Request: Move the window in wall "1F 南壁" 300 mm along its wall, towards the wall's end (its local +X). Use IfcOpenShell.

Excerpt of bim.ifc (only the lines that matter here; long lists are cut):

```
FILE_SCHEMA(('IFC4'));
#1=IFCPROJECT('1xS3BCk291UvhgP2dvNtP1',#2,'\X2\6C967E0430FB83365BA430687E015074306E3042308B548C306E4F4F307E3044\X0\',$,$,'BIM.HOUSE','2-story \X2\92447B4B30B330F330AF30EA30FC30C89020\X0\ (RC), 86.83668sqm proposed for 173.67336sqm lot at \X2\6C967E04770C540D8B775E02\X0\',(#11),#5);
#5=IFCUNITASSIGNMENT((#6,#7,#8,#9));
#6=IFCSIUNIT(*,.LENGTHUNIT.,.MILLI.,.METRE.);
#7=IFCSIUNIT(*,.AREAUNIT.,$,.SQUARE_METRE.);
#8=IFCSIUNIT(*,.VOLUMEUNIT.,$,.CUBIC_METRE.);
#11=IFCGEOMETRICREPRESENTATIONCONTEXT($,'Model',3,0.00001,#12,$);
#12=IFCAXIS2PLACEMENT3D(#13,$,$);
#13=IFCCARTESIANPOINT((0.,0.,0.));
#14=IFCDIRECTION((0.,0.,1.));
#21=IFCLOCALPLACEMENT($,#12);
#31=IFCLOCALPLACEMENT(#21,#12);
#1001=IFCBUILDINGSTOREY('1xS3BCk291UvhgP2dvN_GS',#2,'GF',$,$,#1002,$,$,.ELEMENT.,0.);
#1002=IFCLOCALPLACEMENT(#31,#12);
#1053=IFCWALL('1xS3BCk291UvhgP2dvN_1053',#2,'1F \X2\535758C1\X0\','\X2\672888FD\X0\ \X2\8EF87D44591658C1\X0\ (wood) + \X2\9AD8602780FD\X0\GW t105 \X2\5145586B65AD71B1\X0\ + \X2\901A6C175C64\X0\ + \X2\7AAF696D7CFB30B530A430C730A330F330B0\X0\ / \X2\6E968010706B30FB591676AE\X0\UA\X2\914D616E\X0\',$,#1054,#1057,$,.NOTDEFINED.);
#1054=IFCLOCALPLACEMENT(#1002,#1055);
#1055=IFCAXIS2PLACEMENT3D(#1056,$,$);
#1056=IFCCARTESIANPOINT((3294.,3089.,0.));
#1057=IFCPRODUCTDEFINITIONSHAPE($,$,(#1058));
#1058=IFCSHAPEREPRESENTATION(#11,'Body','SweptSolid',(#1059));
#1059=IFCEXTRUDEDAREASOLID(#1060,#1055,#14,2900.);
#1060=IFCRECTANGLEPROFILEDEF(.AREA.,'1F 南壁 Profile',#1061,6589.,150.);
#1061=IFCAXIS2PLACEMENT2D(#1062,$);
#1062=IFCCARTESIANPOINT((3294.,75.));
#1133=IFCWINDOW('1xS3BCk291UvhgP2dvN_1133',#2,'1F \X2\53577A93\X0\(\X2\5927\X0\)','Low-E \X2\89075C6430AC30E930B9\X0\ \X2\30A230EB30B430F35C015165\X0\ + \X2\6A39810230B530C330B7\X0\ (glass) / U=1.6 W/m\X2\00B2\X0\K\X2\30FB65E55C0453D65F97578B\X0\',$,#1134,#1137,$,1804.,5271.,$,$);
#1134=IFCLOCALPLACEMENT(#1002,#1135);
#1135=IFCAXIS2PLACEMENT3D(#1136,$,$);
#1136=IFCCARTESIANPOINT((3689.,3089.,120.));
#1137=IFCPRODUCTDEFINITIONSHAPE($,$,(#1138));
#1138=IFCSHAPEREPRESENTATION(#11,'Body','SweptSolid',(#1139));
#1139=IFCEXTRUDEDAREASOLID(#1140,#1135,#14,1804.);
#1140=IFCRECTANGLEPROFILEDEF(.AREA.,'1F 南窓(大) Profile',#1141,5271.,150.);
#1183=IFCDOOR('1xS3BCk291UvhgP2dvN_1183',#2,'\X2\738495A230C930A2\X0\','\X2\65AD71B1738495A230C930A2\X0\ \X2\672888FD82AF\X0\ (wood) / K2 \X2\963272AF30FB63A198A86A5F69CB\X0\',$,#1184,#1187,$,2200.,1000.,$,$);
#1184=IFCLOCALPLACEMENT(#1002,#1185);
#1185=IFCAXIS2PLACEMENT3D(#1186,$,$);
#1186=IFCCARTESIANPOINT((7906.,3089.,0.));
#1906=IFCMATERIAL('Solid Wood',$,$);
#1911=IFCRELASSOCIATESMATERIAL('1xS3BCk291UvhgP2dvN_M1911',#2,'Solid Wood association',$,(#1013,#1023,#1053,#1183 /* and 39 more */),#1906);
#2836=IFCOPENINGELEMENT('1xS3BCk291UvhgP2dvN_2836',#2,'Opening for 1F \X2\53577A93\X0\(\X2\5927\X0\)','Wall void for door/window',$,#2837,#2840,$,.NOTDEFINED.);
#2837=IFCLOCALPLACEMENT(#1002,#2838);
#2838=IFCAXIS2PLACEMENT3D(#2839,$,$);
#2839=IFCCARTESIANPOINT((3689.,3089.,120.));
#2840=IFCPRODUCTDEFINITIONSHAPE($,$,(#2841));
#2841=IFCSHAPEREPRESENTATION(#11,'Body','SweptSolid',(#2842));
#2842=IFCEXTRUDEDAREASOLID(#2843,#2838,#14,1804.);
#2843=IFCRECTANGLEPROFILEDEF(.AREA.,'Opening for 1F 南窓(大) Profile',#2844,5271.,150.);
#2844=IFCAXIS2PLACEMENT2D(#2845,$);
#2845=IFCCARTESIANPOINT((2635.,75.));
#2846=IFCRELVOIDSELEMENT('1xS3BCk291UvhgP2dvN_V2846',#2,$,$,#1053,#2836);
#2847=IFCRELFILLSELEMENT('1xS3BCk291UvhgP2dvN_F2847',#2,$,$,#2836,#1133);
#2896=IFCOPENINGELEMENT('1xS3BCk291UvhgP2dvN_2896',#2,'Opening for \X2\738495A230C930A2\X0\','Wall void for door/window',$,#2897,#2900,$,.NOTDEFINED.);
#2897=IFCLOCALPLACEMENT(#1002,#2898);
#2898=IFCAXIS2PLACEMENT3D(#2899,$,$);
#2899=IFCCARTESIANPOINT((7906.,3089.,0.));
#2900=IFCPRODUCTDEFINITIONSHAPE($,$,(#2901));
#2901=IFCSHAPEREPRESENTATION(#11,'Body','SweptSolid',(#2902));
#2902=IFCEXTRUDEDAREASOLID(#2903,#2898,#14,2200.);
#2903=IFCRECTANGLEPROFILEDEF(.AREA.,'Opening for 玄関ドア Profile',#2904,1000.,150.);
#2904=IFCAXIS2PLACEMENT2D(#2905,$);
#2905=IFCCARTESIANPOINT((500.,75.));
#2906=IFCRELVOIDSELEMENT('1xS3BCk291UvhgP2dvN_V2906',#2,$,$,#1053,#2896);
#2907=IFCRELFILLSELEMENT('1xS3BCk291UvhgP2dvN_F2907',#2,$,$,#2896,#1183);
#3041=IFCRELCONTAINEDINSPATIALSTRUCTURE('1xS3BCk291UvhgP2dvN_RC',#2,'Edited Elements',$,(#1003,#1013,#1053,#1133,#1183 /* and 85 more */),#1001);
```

```python
import ifcopenshell
import ifcopenshell.api.geometry
import ifcopenshell.util.placement
import ifcopenshell.util.unit

model = ifcopenshell.open("bim.ifc")
unit_scale = ifcopenshell.util.unit.calculate_unit_scale(model)

window = model.by_guid("1xS3BCk291UvhgP2dvN_1133")
opening = window.FillsVoids[0].RelatingOpeningElement
wall = opening.VoidsElements[0].RelatingBuildingElement

wall_matrix = ifcopenshell.util.placement.get_local_placement(wall.ObjectPlacement)
shift = wall_matrix[:3, 0] * 0.3 / unit_scale
before = ifcopenshell.util.placement.get_local_placement(window.ObjectPlacement)[:3, 3].copy()

# The window is not placed relative to its opening, so move both.
for product in (opening, window):
    matrix = ifcopenshell.util.placement.get_local_placement(product.ObjectPlacement)
    matrix[:3, 3] += shift
    ifcopenshell.api.geometry.edit_object_placement(model, product=product, matrix=matrix, is_si=False)

after = ifcopenshell.util.placement.get_local_placement(window.ObjectPlacement)[:3, 3]
print("window moved by", (after - before).round(3) + 0.0)

model.write("bim_rev.ifc")
```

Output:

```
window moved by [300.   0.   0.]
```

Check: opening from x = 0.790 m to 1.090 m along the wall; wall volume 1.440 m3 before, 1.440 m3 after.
